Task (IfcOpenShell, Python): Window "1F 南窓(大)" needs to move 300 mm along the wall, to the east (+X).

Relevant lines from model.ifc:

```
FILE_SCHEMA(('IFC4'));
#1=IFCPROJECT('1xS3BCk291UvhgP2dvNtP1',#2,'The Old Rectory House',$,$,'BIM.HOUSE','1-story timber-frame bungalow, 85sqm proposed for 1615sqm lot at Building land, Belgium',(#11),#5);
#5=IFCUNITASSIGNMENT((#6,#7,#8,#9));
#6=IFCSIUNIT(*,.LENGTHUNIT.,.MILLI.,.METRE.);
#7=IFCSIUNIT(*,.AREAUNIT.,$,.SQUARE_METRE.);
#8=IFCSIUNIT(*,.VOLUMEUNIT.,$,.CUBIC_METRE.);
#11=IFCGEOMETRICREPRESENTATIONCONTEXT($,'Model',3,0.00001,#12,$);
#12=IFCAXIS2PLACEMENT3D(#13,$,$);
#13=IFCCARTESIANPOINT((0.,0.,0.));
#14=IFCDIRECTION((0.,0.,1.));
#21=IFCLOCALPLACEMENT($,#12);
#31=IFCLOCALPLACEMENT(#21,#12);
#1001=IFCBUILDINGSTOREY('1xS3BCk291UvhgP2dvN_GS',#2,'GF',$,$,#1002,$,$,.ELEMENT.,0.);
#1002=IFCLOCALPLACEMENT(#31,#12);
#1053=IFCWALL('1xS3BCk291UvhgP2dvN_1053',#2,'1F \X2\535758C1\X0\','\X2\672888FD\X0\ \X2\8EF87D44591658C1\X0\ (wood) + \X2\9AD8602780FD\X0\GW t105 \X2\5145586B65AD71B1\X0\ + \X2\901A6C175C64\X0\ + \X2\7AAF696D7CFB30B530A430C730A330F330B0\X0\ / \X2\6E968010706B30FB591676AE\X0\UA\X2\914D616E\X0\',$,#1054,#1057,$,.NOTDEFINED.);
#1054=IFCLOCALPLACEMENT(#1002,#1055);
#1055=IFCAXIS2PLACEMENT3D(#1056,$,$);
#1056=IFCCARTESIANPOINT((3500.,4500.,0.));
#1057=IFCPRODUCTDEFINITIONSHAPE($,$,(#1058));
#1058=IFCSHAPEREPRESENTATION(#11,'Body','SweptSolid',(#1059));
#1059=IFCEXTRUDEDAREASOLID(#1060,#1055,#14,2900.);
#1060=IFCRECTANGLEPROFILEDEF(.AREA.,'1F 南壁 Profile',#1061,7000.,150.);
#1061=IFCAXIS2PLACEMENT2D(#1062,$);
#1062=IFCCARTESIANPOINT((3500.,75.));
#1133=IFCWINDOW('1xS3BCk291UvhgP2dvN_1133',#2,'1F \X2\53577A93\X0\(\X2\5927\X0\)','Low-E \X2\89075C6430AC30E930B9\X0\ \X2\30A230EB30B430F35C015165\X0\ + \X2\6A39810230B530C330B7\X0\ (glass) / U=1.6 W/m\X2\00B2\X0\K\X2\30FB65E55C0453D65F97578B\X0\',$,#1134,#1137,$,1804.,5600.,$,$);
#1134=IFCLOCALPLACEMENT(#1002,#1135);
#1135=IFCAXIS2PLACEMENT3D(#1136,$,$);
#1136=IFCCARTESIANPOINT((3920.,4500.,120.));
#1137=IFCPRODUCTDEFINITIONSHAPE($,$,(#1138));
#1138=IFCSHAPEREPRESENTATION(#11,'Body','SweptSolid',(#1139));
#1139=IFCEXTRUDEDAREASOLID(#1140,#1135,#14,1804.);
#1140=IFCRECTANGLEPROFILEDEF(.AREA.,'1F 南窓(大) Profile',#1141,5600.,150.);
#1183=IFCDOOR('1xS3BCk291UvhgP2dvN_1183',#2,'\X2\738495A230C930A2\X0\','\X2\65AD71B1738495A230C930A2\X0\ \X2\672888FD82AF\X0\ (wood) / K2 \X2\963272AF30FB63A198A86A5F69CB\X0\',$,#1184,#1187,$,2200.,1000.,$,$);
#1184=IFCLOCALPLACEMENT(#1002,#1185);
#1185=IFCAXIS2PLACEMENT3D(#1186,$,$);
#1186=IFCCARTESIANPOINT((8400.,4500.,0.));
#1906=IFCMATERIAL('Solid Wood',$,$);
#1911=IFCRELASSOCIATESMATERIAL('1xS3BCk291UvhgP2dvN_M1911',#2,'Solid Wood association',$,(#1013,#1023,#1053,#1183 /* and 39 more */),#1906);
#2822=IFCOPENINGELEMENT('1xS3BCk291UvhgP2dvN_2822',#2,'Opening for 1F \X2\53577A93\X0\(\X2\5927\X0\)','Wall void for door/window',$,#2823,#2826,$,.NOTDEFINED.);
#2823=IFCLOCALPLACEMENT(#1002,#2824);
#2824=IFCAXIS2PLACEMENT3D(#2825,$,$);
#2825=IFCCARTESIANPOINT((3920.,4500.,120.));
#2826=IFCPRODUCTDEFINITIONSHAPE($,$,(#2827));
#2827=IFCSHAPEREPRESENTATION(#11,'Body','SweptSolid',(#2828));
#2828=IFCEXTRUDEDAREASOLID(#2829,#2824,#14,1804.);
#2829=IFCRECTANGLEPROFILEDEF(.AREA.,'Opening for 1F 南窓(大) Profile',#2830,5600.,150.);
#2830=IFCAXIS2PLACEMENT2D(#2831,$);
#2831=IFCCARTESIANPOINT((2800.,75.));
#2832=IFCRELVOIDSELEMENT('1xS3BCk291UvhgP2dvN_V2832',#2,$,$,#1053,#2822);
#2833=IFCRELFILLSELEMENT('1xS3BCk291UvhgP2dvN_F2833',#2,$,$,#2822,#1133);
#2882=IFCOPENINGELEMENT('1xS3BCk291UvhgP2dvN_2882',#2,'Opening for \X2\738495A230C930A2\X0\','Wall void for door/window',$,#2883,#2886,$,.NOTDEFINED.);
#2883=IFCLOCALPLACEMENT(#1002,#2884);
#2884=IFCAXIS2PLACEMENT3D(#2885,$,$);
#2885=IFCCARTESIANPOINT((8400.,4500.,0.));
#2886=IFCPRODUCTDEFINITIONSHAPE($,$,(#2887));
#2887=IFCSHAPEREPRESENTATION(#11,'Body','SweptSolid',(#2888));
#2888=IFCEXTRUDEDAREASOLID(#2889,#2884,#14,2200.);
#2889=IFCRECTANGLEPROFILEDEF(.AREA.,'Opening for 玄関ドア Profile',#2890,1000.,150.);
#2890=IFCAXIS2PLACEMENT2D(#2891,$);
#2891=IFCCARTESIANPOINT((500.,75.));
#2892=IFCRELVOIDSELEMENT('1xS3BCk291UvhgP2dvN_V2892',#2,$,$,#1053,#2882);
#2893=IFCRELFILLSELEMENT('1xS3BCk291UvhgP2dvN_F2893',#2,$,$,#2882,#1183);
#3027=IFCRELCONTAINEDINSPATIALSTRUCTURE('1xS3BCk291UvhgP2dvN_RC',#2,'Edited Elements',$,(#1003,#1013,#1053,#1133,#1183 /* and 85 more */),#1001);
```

```python
import ifcopenshell
import ifcopenshell.api.geometry
import ifcopenshell.util.placement
import ifcopenshell.util.unit

model = ifcopenshell.open("model.ifc")
unit_scale = ifcopenshell.util.unit.calculate_unit_scale(model)

window = model.by_id(1133)
opening = window.FillsVoids[0].RelatingOpeningElement
wall = opening.VoidsElements[0].RelatingBuildingElement

wall_matrix = ifcopenshell.util.placement.get_local_placement(wall.ObjectPlacement)
shift = wall_matrix[:3, 0] * 0.3 / unit_scale
before = ifcopenshell.util.placement.get_local_placement(window.ObjectPlacement)[:3, 3].copy()

# The window is not placed relative to its opening, so move both.
for product in (opening, window):
    matrix = ifcopenshell.util.placement.get_local_placement(product.ObjectPlacement)
    matrix[:3, 3] += shift
    ifcopenshell.api.geometry.edit_object_placement(model, product=product, matrix=matrix, is_si=False)

after = ifcopenshell.util.placement.get_local_placement(window.ObjectPlacement)[:3, 3]
print("window moved by", (after - before).round(3) + 0.0)

model.write("model_rev.ifc")
```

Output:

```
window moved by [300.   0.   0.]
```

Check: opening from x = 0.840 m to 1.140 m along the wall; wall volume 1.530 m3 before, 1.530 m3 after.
